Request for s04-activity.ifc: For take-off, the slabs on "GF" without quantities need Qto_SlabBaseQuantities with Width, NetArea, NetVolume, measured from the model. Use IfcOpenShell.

First a look at what the model holds.

```python
import ifcopenshell
import ifcopenshell.util.element
import ifcopenshell.util.unit

model = ifcopenshell.open("s04-activity.ifc")
print(model.schema)
for unit_type in ("LENGTHUNIT", "AREAUNIT", "VOLUMEUNIT"):
    print(unit_type, ifcopenshell.util.unit.calculate_unit_scale(model, unit_type))
storey = next(s for s in model.by_type("IfcBuildingStorey") if s.Name == "GF")
slabs = [e for e in ifcopenshell.util.element.get_decomposition(storey) if e.is_a("IfcSlab")]
for e in sorted(slabs, key=lambda e: e.id()):
    print(e.id(), e.is_a(), e.Name, list(ifcopenshell.util.element.get_psets(e, qtos_only=True)), sep=" | ")
```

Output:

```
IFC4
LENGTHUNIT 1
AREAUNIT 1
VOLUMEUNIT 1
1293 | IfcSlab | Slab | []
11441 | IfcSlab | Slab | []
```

```python
import ifcopenshell
import ifcopenshell.api.pset
import ifcopenshell.geom
import ifcopenshell.util.element
import ifcopenshell.util.shape
import ifcopenshell.util.unit

model = ifcopenshell.open("s04-activity.ifc")
unit_scale = ifcopenshell.util.unit.calculate_unit_scale(model)
area_scale = ifcopenshell.util.unit.calculate_unit_scale(model, "AREAUNIT")
volume_scale = ifcopenshell.util.unit.calculate_unit_scale(model, "VOLUMEUNIT")
settings = ifcopenshell.geom.settings()

storey = next(s for s in model.by_type("IfcBuildingStorey") if s.Name == "GF")
slabs = [e for e in ifcopenshell.util.element.get_decomposition(storey) if e.is_a("IfcSlab")]

for e in sorted(slabs, key=lambda e: e.id()):
    if ifcopenshell.util.element.get_psets(e, qtos_only=True, should_inherit=False):
        continue
    # Geometry comes back in metres, in the element's own axes.
    shape = ifcopenshell.geom.create_shape(settings, e)
    values = {
        "Width": ifcopenshell.util.shape.get_z(shape.geometry) / unit_scale,
        "NetArea": ifcopenshell.util.shape.get_footprint_area(shape.geometry) / area_scale,
        "NetVolume": ifcopenshell.util.shape.get_volume(shape.geometry) / volume_scale,
    }
    qto = ifcopenshell.api.pset.add_qto(model, product=e, name="Qto_SlabBaseQuantities")
    ifcopenshell.api.pset.edit_qto(model, qto=qto, properties=values)
    print(e.id(), {k: round(v, 3) for k, v in values.items()})

model.write("s04-activity_edited.ifc")
```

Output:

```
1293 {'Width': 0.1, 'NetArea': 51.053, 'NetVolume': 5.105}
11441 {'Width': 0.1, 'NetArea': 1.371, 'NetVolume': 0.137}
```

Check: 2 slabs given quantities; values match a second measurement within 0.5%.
